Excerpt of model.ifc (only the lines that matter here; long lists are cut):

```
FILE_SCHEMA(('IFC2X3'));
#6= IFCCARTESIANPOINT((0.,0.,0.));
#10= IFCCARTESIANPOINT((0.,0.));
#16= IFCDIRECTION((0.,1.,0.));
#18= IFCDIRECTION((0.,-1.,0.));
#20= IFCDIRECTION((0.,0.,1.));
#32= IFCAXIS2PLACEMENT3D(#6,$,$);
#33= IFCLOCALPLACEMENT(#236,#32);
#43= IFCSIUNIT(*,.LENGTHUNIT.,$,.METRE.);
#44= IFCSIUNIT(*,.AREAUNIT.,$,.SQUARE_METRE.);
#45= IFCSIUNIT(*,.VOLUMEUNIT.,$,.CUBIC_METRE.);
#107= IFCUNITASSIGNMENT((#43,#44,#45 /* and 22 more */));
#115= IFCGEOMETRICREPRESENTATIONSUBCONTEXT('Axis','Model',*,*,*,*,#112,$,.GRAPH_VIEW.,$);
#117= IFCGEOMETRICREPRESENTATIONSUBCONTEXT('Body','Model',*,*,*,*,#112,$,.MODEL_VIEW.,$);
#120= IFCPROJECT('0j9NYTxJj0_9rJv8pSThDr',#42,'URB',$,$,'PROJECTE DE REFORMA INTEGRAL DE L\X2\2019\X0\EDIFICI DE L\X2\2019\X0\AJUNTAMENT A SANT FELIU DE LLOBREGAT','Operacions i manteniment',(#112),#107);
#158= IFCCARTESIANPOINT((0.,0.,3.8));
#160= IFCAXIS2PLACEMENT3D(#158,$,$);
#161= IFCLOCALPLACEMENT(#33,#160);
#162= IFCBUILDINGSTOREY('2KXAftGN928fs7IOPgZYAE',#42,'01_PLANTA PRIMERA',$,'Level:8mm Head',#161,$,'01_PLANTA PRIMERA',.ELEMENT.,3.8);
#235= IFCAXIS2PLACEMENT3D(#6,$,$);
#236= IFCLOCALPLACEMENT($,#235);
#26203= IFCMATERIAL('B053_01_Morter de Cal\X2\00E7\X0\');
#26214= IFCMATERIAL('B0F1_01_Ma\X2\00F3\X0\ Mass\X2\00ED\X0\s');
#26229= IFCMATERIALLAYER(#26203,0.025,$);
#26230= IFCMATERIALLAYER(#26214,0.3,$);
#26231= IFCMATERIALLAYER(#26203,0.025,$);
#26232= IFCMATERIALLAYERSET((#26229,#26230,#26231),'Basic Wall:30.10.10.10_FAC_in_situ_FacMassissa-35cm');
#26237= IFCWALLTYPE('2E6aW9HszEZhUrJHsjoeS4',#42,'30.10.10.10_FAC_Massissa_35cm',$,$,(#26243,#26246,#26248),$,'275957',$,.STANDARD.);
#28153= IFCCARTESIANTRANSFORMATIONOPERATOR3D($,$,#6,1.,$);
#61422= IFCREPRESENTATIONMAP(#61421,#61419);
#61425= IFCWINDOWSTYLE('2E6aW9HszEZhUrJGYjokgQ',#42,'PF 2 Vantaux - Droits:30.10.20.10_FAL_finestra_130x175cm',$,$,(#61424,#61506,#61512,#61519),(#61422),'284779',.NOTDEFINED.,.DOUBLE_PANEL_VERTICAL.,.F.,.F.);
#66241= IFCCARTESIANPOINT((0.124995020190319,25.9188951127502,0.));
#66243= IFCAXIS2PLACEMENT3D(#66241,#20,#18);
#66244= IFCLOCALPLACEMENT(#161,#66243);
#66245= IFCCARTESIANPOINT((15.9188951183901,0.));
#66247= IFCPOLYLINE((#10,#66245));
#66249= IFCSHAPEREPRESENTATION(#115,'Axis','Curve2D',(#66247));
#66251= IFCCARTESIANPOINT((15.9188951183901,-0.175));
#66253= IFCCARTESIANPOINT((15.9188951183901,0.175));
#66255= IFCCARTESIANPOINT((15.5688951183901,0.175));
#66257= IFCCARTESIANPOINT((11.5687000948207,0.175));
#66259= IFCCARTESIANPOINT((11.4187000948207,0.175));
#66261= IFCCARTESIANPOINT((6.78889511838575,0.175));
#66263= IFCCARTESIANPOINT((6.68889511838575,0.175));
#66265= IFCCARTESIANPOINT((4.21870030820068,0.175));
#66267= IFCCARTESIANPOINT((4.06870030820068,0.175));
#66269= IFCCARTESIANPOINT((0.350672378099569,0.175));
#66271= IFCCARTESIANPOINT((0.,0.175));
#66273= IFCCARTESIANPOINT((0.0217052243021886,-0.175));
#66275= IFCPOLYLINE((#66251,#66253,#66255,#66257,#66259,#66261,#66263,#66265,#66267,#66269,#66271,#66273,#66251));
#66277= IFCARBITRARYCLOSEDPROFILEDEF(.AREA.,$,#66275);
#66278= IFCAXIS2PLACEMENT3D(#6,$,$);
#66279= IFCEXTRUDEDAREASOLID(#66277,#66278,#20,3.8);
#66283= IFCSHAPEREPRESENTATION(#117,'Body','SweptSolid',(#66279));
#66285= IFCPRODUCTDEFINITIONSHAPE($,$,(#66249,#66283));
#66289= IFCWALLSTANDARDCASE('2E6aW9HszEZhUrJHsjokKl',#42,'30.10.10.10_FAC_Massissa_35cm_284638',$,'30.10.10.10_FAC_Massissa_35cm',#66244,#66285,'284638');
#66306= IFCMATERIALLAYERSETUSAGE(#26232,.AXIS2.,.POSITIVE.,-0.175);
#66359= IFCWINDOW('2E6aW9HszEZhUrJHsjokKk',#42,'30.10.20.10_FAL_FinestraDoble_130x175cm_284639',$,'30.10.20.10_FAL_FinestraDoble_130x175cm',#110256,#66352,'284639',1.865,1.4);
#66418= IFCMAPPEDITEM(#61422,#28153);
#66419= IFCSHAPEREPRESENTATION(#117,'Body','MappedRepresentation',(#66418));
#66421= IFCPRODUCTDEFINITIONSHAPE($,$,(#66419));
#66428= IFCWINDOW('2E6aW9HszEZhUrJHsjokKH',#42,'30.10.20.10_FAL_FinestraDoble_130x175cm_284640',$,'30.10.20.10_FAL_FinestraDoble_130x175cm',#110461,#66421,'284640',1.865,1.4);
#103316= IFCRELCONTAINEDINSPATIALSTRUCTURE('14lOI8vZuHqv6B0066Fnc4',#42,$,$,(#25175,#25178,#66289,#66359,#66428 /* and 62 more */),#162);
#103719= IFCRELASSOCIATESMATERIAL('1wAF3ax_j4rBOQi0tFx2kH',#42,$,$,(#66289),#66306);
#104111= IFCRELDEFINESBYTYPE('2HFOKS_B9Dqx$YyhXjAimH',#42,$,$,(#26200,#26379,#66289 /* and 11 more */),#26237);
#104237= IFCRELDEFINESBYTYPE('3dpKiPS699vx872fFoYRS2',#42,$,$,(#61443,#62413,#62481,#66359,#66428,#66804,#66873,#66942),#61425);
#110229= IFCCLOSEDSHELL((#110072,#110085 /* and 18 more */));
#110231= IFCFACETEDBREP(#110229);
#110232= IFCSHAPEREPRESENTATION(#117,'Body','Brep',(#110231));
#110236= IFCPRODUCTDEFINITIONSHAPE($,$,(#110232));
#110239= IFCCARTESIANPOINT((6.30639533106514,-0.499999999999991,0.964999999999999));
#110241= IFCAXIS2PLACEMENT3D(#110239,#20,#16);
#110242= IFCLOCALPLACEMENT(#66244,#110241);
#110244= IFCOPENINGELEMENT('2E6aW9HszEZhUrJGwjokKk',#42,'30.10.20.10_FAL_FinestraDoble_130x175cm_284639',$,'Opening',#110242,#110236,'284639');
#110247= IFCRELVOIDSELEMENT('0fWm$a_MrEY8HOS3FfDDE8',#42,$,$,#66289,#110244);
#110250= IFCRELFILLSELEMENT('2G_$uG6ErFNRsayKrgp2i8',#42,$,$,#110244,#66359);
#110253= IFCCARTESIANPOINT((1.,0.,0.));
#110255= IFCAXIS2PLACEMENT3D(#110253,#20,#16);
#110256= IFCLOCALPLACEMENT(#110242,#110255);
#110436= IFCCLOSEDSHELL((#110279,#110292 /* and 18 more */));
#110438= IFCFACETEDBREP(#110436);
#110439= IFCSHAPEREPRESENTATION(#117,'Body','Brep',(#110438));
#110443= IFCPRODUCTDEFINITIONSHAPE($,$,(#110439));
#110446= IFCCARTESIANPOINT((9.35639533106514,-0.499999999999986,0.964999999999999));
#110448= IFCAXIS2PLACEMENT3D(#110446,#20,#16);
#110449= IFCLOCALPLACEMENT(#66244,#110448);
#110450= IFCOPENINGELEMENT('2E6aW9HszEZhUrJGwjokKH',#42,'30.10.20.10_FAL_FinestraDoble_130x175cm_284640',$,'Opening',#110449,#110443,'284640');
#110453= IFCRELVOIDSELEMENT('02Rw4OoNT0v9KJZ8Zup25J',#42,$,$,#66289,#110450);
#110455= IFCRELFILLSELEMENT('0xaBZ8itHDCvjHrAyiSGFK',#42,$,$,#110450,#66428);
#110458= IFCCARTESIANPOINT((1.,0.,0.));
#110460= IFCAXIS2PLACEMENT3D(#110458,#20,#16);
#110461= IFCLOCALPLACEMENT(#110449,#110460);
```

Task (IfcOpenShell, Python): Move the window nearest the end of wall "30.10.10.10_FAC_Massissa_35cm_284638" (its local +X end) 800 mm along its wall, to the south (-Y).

```python
import ifcopenshell
import ifcopenshell.api.geometry
import ifcopenshell.util.placement
import ifcopenshell.util.unit

model = ifcopenshell.open("model.ifc")
unit_scale = ifcopenshell.util.unit.calculate_unit_scale(model)

window = model.by_guid("2E6aW9HszEZhUrJHsjokKH")
opening = window.FillsVoids[0].RelatingOpeningElement
wall = opening.VoidsElements[0].RelatingBuildingElement

wall_matrix = ifcopenshell.util.placement.get_local_placement(wall.ObjectPlacement)
shift = wall_matrix[:3, 0] * 0.8 / unit_scale
before = ifcopenshell.util.placement.get_local_placement(window.ObjectPlacement)[:3, 3].copy()

# The window is placed relative to its opening, so it follows when the opening moves.
matrix = ifcopenshell.util.placement.get_local_placement(opening.ObjectPlacement)
matrix[:3, 3] += shift
ifcopenshell.api.geometry.edit_object_placement(
    model, product=opening, matrix=matrix, is_si=False, should_transform_children=True
)

after = ifcopenshell.util.placement.get_local_placement(window.ObjectPlacement)[:3, 3]
print("window moved by", (after - before).round(3) + 0.0)

model.write("model_v2.ifc")
```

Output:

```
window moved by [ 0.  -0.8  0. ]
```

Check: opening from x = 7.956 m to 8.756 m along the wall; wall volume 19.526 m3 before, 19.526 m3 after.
